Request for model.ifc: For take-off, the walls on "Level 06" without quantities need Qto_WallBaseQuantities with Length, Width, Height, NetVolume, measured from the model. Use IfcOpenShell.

First a look at what the model holds.

```python
import ifcopenshell
import ifcopenshell.util.element
import ifcopenshell.util.unit

model = ifcopenshell.open("model.ifc")
print(model.schema)
for unit_type in ("LENGTHUNIT", "AREAUNIT", "VOLUMEUNIT"):
    print(unit_type, ifcopenshell.util.unit.calculate_unit_scale(model, unit_type))
storey = next(s for s in model.by_type("IfcBuildingStorey") if s.Name == "Level 06")
walls = [e for e in ifcopenshell.util.element.get_decomposition(storey) if e.is_a("IfcWall")]
for e in sorted(walls, key=lambda e: e.id()):
    print(e.id(), e.is_a(), e.Name, list(ifcopenshell.util.element.get_psets(e, qtos_only=True)), sep=" | ")
```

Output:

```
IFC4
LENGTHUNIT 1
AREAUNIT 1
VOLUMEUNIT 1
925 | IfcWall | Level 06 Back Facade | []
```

```python
import ifcopenshell
import ifcopenshell.api.pset
import ifcopenshell.geom
import ifcopenshell.util.element
import ifcopenshell.util.shape
import ifcopenshell.util.unit

model = ifcopenshell.open("model.ifc")
unit_scale = ifcopenshell.util.unit.calculate_unit_scale(model)
volume_scale = ifcopenshell.util.unit.calculate_unit_scale(model, "VOLUMEUNIT")
settings = ifcopenshell.geom.settings()

storey = next(s for s in model.by_type("IfcBuildingStorey") if s.Name == "Level 06")
walls = [e for e in ifcopenshell.util.element.get_decomposition(storey) if e.is_a("IfcWall")]

for e in sorted(walls, key=lambda e: e.id()):
    if ifcopenshell.util.element.get_psets(e, qtos_only=True, should_inherit=False):
        continue
    # Geometry comes back in metres, in the element's own axes.
    shape = ifcopenshell.geom.create_shape(settings, e)
    values = {
        "Length": ifcopenshell.util.shape.get_x(shape.geometry) / unit_scale,
        "Width": ifcopenshell.util.shape.get_y(shape.geometry) / unit_scale,
        "Height": ifcopenshell.util.shape.get_z(shape.geometry) / unit_scale,
        "NetVolume": ifcopenshell.util.shape.get_volume(shape.geometry) / volume_scale,
    }
    qto = ifcopenshell.api.pset.add_qto(model, product=e, name="Qto_WallBaseQuantities")
    ifcopenshell.api.pset.edit_qto(model, qto=qto, properties=values)
    print(e.id(), {k: round(v, 3) for k, v in values.items()})

model.write("model_v2.ifc")
```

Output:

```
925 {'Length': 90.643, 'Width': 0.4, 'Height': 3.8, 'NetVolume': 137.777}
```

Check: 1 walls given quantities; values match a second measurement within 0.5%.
